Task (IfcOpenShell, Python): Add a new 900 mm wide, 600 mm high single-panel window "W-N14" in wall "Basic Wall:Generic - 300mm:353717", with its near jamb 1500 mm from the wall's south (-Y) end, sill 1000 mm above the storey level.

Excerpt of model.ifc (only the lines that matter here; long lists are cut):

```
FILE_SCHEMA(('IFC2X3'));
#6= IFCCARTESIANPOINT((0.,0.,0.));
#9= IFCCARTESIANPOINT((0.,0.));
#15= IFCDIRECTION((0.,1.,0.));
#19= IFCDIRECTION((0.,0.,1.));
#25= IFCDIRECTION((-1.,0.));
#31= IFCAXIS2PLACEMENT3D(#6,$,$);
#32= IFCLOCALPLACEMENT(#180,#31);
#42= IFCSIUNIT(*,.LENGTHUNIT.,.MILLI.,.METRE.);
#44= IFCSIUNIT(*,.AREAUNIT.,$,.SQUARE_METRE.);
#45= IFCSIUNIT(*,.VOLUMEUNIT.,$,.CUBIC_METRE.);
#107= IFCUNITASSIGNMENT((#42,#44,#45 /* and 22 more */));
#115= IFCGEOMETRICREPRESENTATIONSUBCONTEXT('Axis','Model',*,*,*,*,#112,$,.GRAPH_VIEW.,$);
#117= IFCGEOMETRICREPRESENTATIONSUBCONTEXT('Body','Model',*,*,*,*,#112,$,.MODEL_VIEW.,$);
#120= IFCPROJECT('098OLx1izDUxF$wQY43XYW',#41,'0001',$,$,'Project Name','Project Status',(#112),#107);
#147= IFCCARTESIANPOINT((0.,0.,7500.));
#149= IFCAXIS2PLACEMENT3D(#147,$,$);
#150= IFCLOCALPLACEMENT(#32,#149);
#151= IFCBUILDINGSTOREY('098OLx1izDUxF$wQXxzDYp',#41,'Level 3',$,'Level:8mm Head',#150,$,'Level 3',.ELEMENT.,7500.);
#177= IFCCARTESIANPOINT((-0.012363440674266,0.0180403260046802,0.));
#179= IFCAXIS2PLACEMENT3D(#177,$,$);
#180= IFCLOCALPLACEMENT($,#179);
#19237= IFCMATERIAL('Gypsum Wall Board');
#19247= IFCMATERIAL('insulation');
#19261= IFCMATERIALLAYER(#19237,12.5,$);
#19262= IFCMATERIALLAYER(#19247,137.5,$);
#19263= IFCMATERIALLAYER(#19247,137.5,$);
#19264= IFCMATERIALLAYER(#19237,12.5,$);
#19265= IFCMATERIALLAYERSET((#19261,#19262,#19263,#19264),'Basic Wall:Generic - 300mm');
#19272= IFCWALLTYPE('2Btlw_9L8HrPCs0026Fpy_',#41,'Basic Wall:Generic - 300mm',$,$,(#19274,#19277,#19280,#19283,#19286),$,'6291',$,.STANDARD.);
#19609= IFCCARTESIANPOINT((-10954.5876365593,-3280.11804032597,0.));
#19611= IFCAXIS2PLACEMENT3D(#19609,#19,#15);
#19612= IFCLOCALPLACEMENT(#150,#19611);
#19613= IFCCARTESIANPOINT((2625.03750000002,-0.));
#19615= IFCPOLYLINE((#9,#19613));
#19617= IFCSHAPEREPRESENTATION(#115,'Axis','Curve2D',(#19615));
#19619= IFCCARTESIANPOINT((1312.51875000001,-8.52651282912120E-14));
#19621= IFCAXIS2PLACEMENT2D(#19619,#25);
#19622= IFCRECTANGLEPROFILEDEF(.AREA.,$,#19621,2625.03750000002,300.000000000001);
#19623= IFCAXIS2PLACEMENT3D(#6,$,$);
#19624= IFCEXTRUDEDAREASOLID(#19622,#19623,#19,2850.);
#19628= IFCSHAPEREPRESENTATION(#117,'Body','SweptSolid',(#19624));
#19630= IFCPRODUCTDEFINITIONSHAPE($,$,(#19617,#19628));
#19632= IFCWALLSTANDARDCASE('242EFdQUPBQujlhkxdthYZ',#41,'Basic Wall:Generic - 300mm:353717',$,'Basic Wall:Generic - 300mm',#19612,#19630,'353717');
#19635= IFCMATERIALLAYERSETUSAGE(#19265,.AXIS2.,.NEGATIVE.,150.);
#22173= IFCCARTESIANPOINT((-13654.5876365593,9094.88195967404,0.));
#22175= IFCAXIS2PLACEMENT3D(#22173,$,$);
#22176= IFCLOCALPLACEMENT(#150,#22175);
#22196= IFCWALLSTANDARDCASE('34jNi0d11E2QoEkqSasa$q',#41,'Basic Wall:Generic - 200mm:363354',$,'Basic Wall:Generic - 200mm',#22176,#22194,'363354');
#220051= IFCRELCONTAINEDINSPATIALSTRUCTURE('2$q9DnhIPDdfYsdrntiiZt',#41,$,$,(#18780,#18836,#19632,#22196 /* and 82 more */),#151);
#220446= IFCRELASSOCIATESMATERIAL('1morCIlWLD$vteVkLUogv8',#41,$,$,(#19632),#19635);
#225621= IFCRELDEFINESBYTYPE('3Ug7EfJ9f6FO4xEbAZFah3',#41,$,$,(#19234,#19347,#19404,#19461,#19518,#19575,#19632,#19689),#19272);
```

```python
import numpy as np
import ifcopenshell
import ifcopenshell.api.feature
import ifcopenshell.api.geometry
import ifcopenshell.api.root
import ifcopenshell.api.spatial
import ifcopenshell.api.type
import ifcopenshell.geom
import ifcopenshell.util.element
import ifcopenshell.util.placement
import ifcopenshell.util.representation
import ifcopenshell.util.shape
import ifcopenshell.util.unit

model = ifcopenshell.open("model.ifc")
unit_scale = ifcopenshell.util.unit.calculate_unit_scale(model)
settings = ifcopenshell.geom.settings()


def volume(element):
    """Net volume in cubic metres, openings subtracted."""
    shape = ifcopenshell.geom.create_shape(settings, element)
    return ifcopenshell.util.shape.get_volume(shape.geometry)


wall = model.by_guid("242EFdQUPBQujlhkxdthYZ")
storey = ifcopenshell.util.element.get_container(wall, ifc_class="IfcBuildingStorey")
context = ifcopenshell.util.representation.get_context(model, "Model", "Body", "MODEL_VIEW")
before = volume(wall)

width, height, from_end, sill = 0.9, 0.6, 1.5, 1  # metres

# The wall runs along its own X axis, and the end named is its -X end.
wall_shape = ifcopenshell.geom.create_shape(settings, wall)
x, y, z = ifcopenshell.util.shape.get_vertices(wall_shape.geometry).T
start = x.min() + from_end
face, thickness = float(y.min()), float(y.max() - y.min())
wall_matrix = ifcopenshell.util.placement.get_local_placement(wall.ObjectPlacement)
level = ifcopenshell.util.placement.get_local_placement(storey.ObjectPlacement)[2, 3]


def in_wall(x, y):
    """Placement at x, y metres in the wall's axes, at sill height."""
    matrix = wall_matrix.copy()
    matrix[:, 3] = wall_matrix @ np.array([x / unit_scale, y / unit_scale, 0.0, 1.0])
    matrix[2, 3] = level + sill / unit_scale
    return matrix


# Opening: a box that overshoots both wall faces by 50 mm.
opening = ifcopenshell.api.root.create_entity(model, ifc_class="IfcOpeningElement")
box = ifcopenshell.api.geometry.add_wall_representation(
    model, context=context, length=width, height=height, thickness=thickness + 0.1
)
ifcopenshell.api.geometry.assign_representation(model, product=opening, representation=box)
ifcopenshell.api.geometry.edit_object_placement(model, product=opening, matrix=in_wall(start, face - 0.05), is_si=False)
ifcopenshell.api.feature.add_feature(model, feature=opening, element=wall)

window = ifcopenshell.api.root.create_entity(model, ifc_class="IfcWindow", name="W-N14")
window.OverallWidth, window.OverallHeight = width / unit_scale, height / unit_scale
body = ifcopenshell.api.geometry.add_window_representation(
    model,
    context=context,
    overall_width=window.OverallWidth,
    overall_height=window.OverallHeight,
    partition_type="SINGLE_PANEL",
)
ifcopenshell.api.geometry.assign_representation(model, product=window, representation=body)
ifcopenshell.api.spatial.assign_container(model, products=[window], relating_structure=storey)
fills = ifcopenshell.api.feature.add_filling(model, opening=opening, element=window)
fills.OwnerHistory = window.OwnerHistory  # required in IFC2X3

# IFC2X3 keeps the operation on the window style.
style = ifcopenshell.api.root.create_entity(model, ifc_class="IfcWindowStyle", name="W-N14")
style.OperationType, style.ConstructionType = "SINGLE_PANEL", "NOTDEFINED"
style.ParameterTakesPrecedence = style.Sizeable = False
ifcopenshell.api.type.assign_type(model, related_objects=[window], relating_type=style)

# Centre the window in the wall's thickness.
ifcopenshell.api.geometry.edit_object_placement(model, product=window, matrix=in_wall(start, face), is_si=False)
window_shape = ifcopenshell.geom.create_shape(settings, window)
depth = ifcopenshell.util.shape.get_vertices(window_shape.geometry)[:, 1]
offset = face + thickness / 2 - (depth.min() + depth.max()) / 2
ifcopenshell.api.geometry.edit_object_placement(model, product=window, matrix=in_wall(start, offset), is_si=False)

after = volume(wall)

print(f"wall volume {before:.3f} -> {after:.3f} m3")

model.write("model_rev.ifc")
```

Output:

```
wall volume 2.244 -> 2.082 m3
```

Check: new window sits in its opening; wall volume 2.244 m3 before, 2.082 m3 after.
